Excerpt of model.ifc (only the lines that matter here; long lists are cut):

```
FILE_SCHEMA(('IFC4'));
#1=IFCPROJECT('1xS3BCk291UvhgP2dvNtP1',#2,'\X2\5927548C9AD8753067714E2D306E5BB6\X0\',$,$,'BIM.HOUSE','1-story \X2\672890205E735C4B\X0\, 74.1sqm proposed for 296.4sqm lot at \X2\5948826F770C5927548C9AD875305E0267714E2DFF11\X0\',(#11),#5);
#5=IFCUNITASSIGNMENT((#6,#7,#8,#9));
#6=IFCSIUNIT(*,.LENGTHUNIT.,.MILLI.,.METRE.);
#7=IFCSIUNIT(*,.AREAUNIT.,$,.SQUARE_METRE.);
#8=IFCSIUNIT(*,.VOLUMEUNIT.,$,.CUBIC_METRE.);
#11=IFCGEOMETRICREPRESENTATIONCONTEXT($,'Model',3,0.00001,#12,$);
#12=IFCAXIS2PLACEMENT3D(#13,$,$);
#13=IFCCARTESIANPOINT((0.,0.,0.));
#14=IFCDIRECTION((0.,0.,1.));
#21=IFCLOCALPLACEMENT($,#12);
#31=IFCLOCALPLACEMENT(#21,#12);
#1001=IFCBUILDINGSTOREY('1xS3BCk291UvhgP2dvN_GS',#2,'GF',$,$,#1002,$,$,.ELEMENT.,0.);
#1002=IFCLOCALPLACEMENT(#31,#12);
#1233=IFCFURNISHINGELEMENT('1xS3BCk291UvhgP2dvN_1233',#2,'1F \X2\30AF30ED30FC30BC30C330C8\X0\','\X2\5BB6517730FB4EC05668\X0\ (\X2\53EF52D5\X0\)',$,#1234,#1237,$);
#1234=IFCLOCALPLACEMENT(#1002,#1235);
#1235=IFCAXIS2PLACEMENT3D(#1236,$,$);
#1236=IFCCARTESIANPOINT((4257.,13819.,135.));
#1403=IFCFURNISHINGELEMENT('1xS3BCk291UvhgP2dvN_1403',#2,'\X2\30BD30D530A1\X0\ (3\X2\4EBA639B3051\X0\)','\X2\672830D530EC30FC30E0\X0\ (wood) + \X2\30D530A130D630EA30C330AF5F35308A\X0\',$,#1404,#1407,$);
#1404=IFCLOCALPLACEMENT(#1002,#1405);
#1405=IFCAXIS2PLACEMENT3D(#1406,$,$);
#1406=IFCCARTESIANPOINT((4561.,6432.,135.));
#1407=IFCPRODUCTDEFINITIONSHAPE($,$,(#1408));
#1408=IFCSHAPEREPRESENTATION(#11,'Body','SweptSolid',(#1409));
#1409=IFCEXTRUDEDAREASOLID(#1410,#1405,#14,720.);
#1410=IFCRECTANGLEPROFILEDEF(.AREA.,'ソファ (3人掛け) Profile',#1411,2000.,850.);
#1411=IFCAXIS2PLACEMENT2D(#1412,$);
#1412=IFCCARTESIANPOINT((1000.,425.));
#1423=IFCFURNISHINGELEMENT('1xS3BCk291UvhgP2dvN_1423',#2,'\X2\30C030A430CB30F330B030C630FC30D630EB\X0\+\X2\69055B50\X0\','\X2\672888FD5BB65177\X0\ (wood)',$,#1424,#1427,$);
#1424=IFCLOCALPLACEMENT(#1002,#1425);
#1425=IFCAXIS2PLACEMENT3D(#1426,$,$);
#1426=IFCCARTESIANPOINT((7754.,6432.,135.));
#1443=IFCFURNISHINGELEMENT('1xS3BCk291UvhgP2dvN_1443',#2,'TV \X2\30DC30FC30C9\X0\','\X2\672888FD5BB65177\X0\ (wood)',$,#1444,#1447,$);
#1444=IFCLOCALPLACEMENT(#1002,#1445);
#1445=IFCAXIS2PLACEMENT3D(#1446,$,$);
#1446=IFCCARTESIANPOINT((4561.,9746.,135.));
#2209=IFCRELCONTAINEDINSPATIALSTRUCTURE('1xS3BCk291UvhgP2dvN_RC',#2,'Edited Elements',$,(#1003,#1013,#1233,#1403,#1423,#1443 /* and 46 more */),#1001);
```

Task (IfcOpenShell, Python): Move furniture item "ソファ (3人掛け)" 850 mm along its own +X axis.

```python
import ifcopenshell
import ifcopenshell.api.geometry
import ifcopenshell.util.placement
import ifcopenshell.util.unit

model = ifcopenshell.open("model.ifc")
unit_scale = ifcopenshell.util.unit.calculate_unit_scale(model)

item = model.by_guid("1xS3BCk291UvhgP2dvN_1403")
matrix = ifcopenshell.util.placement.get_local_placement(item.ObjectPlacement)
matrix[:3, 3] += matrix[:3, 0] * 0.85 / unit_scale
ifcopenshell.api.geometry.edit_object_placement(model, product=item, matrix=matrix, is_si=False)

print(ifcopenshell.util.placement.get_local_placement(item.ObjectPlacement).round(3) + 0.0)

model.write("model_v2.ifc")
```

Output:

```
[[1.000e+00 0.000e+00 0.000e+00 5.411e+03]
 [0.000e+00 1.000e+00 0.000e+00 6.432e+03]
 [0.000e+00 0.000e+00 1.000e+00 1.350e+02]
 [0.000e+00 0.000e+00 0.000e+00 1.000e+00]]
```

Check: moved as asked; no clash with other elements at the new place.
